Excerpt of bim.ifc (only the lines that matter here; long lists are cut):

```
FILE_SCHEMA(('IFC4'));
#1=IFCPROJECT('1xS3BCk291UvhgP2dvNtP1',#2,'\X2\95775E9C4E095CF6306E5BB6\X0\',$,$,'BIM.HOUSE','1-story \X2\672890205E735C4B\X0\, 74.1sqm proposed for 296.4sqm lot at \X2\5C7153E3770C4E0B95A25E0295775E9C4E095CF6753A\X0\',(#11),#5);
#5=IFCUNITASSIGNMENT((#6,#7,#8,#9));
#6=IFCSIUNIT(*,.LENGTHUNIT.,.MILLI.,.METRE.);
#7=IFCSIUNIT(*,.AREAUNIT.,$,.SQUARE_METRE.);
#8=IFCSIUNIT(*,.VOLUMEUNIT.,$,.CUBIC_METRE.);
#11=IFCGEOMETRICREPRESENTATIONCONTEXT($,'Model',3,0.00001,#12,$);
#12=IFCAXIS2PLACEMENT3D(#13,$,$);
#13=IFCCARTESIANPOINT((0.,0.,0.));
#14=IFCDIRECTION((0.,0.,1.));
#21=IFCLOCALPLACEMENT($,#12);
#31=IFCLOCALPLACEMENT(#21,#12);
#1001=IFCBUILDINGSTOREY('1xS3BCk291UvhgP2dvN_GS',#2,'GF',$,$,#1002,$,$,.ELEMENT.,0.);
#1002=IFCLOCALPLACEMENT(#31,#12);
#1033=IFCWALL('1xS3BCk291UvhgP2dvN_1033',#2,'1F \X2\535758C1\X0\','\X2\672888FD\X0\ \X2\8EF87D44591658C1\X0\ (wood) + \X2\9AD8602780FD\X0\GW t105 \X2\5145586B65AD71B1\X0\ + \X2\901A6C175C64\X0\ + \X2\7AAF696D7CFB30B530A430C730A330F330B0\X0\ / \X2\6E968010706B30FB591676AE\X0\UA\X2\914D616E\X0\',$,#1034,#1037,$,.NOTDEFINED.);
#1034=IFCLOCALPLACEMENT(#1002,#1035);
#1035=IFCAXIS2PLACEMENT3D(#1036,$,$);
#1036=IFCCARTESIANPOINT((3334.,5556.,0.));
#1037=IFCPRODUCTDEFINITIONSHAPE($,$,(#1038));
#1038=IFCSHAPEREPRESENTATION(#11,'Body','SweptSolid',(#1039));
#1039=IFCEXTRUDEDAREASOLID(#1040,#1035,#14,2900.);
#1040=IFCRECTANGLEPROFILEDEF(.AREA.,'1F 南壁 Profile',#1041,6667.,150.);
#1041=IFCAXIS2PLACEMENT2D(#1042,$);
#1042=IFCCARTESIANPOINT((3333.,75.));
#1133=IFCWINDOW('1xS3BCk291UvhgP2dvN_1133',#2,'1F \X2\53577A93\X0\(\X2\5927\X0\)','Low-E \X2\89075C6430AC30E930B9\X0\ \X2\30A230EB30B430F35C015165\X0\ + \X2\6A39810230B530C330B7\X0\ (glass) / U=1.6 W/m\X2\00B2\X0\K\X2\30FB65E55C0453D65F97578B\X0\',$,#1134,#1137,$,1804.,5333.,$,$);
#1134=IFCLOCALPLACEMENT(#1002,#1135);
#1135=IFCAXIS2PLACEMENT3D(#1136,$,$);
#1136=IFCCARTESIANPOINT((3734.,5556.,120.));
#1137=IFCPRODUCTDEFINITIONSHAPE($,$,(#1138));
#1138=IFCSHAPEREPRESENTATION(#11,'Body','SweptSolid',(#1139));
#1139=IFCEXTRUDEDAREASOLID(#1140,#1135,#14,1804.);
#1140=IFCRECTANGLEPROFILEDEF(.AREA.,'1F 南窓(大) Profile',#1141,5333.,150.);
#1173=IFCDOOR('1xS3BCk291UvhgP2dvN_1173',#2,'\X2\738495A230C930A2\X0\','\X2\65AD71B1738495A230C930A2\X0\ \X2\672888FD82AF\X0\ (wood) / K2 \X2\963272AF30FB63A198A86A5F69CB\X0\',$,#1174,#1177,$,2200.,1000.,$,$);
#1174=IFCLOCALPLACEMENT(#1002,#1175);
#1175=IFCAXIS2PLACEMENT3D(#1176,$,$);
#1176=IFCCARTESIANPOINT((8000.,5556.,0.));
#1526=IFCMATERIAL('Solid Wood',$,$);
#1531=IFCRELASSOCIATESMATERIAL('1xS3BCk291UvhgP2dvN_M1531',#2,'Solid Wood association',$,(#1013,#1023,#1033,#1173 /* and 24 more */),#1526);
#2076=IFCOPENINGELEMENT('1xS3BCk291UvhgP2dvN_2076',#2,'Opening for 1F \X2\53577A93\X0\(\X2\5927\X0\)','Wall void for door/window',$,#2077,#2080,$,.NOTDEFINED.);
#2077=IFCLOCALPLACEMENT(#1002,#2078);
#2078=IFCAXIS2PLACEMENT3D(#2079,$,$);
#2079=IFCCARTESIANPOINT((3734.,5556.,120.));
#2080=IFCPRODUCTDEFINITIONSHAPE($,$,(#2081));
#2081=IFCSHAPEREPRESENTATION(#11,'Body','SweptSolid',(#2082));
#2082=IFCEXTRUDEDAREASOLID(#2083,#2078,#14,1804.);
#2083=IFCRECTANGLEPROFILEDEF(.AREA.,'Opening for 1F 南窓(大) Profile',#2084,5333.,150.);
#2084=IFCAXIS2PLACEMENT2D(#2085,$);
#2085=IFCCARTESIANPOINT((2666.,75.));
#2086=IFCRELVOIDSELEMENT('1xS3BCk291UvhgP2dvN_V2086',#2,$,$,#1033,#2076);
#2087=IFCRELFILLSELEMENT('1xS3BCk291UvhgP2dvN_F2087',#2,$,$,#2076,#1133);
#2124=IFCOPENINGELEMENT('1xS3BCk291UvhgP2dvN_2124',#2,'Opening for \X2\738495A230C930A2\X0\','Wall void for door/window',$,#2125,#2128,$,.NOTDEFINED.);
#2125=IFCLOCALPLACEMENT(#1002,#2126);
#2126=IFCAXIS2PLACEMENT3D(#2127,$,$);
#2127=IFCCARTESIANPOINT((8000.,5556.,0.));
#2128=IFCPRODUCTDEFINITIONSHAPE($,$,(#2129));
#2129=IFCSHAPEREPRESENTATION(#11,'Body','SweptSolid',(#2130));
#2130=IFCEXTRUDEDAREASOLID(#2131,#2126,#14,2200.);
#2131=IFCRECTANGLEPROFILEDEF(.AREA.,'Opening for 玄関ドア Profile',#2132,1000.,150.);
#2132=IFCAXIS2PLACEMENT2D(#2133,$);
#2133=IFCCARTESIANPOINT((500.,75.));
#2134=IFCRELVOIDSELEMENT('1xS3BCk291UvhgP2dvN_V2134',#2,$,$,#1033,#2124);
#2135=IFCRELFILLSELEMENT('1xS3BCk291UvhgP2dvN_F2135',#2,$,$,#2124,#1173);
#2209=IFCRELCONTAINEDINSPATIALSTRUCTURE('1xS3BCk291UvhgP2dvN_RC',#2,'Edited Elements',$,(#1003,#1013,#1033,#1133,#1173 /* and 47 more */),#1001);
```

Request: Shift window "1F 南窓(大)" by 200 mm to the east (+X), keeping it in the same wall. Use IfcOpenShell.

```python
import ifcopenshell
import ifcopenshell.api.geometry
import ifcopenshell.util.placement

model = ifcopenshell.open("bim.ifc")

window = model.by_guid("1xS3BCk291UvhgP2dvN_1133")
opening = window.FillsVoids[0].RelatingOpeningElement
wall = opening.VoidsElements[0].RelatingBuildingElement

wall_matrix = ifcopenshell.util.placement.get_local_placement(wall.ObjectPlacement)
shift = wall_matrix[:3, 0] * 200.0
before = ifcopenshell.util.placement.get_local_placement(window.ObjectPlacement)[:3, 3].copy()

# The window is not placed relative to its opening, so move both.
for product in (opening, window):
    matrix = ifcopenshell.util.placement.get_local_placement(product.ObjectPlacement)
    matrix[:3, 3] += shift
    ifcopenshell.api.geometry.edit_object_placement(model, product=product, matrix=matrix, is_si=False)

after = ifcopenshell.util.placement.get_local_placement(window.ObjectPlacement)[:3, 3]
print("window moved by", (after - before).round(3) + 0.0)

model.write("bim-out.ifc")
```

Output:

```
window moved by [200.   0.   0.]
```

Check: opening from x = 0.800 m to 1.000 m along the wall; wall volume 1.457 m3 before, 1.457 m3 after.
